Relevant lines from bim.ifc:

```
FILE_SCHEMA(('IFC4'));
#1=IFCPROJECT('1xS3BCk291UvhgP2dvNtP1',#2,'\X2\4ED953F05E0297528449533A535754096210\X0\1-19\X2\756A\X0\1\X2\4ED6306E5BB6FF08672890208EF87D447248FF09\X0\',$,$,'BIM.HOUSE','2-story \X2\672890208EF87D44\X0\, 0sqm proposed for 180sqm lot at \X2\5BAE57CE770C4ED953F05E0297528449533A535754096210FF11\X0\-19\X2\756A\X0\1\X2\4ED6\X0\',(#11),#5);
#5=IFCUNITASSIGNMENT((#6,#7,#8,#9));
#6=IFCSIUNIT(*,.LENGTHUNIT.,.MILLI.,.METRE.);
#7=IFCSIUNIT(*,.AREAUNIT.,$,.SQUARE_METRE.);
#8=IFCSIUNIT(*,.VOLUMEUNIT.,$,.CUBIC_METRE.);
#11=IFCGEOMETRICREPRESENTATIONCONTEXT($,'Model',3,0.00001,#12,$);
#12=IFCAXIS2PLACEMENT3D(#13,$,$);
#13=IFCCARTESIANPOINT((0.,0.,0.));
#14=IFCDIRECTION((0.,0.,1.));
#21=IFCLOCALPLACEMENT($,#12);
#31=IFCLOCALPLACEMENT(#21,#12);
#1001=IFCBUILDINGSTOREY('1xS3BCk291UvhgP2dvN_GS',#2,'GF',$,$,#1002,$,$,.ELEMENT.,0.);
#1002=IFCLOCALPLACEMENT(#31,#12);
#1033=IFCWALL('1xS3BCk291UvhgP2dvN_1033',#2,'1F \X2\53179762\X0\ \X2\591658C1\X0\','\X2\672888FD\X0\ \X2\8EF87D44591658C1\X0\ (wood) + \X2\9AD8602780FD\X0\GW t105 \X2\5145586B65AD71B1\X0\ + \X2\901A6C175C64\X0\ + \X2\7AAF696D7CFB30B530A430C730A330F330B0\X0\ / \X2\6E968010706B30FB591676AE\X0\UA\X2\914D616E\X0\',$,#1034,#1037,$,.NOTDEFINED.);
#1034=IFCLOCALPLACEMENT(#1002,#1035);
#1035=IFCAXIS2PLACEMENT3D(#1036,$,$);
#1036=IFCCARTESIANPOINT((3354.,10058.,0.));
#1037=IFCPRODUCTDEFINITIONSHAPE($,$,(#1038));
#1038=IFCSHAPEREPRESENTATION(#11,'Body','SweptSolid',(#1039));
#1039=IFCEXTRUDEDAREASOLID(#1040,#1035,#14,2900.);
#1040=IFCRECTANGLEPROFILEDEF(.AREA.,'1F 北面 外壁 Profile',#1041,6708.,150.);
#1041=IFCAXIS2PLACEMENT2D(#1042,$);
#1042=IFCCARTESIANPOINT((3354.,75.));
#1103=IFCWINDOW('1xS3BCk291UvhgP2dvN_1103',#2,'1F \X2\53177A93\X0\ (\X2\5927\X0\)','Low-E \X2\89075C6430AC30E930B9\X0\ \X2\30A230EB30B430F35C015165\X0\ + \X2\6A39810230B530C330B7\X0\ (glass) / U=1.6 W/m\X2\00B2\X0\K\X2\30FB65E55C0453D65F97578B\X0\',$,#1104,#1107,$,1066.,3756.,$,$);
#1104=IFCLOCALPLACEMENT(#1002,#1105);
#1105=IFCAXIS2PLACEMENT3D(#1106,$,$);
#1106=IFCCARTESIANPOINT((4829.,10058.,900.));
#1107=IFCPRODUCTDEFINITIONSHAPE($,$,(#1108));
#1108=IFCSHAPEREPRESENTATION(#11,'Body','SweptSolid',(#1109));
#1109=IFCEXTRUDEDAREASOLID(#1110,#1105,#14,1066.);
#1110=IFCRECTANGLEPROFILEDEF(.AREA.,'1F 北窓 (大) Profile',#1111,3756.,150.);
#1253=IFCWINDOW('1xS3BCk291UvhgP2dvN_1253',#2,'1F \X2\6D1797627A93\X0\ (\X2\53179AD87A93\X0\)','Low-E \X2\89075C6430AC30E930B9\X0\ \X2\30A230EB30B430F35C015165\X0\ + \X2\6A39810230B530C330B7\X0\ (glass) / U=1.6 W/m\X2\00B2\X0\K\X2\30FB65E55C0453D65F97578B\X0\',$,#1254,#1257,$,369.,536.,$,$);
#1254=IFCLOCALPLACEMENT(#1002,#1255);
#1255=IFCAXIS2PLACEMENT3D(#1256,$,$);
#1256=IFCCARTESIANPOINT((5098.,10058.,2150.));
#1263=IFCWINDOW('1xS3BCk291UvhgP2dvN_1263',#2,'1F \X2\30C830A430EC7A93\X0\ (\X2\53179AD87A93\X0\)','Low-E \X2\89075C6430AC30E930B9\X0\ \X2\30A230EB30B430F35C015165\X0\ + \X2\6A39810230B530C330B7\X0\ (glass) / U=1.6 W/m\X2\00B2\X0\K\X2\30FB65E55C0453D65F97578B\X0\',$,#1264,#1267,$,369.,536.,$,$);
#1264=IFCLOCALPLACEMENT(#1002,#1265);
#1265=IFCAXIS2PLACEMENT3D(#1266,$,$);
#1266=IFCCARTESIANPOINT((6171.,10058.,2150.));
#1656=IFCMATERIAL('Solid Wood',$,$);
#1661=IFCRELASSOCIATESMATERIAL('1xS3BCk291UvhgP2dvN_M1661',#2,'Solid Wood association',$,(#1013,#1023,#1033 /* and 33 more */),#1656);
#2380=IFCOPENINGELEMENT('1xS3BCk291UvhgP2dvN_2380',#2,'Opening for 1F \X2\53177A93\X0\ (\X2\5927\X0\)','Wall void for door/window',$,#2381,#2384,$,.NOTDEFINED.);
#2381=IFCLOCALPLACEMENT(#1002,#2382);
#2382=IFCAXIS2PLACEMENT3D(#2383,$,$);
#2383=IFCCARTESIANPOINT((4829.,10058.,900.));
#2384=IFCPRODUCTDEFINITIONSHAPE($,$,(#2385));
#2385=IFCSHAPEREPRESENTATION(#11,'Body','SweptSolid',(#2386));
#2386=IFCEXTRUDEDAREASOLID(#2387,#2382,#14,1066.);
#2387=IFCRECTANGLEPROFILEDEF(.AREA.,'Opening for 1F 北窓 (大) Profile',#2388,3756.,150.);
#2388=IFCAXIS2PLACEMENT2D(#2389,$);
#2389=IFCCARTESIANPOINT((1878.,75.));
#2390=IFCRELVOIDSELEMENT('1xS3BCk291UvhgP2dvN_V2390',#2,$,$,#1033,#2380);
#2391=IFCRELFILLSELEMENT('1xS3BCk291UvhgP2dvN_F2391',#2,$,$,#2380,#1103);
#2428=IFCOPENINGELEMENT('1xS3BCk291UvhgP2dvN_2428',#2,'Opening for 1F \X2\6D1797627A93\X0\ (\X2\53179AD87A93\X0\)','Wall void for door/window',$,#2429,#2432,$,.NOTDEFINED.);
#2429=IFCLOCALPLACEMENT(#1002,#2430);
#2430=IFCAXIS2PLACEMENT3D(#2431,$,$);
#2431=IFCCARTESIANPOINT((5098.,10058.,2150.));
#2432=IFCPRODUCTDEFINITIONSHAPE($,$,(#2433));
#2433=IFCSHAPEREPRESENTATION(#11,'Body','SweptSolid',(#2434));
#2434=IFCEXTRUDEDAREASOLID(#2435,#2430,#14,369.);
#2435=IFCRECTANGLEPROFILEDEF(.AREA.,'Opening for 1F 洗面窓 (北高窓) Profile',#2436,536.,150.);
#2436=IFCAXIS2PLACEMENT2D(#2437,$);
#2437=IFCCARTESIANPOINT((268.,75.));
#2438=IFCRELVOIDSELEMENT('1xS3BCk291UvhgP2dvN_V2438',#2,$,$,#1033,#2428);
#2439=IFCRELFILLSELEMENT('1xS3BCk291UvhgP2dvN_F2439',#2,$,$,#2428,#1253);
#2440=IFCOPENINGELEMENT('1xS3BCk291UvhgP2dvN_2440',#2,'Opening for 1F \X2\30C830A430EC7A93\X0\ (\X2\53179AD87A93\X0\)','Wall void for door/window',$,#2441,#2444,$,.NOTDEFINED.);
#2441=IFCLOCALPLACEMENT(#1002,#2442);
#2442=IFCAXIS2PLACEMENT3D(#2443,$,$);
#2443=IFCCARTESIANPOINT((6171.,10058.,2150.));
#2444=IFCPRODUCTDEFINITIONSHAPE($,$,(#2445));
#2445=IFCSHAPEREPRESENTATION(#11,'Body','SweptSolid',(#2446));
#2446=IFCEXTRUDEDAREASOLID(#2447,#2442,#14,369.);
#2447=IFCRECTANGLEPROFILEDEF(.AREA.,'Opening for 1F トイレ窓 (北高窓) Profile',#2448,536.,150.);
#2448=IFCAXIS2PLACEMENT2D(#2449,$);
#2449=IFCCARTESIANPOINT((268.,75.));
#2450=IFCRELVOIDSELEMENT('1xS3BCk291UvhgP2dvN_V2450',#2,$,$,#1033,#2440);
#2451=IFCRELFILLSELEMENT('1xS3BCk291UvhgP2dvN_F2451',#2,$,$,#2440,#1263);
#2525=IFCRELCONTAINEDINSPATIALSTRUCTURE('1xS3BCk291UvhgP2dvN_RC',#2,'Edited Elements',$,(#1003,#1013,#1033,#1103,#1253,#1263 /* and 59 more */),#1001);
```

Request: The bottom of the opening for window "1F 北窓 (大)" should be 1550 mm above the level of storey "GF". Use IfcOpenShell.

```python
import numpy as np
import ifcopenshell
import ifcopenshell.api.geometry
import ifcopenshell.geom
import ifcopenshell.util.element
import ifcopenshell.util.placement
import ifcopenshell.util.shape
import ifcopenshell.util.unit

model = ifcopenshell.open("bim.ifc")
unit_scale = ifcopenshell.util.unit.calculate_unit_scale(model)

window = model.by_id(1103)
opening = window.FillsVoids[0].RelatingOpeningElement
storey = ifcopenshell.util.element.get_container(window, ifc_class="IfcBuildingStorey")
level = ifcopenshell.util.placement.get_local_placement(storey.ObjectPlacement)[2, 3]

# The opening's origin need not be at the sill, so measure its lowest point.
shape = ifcopenshell.geom.create_shape(ifcopenshell.geom.settings(), opening)
bottom = ifcopenshell.util.shape.get_shape_bottom_elevation(shape, shape.geometry) / unit_scale
dz = level + 1.55 / unit_scale - bottom

shift = np.array([0.0, 0.0, dz])
# The window is not placed relative to its opening, so move both.
for product in (opening, window):
    matrix = ifcopenshell.util.placement.get_local_placement(product.ObjectPlacement)
    matrix[:3, 3] += shift
    ifcopenshell.api.geometry.edit_object_placement(model, product=product, matrix=matrix, is_si=False)

print(f"moved by {dz * unit_scale:+.3f} m")

model.write("bim-out.ifc")
```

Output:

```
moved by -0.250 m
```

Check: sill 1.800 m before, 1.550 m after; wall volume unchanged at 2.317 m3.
